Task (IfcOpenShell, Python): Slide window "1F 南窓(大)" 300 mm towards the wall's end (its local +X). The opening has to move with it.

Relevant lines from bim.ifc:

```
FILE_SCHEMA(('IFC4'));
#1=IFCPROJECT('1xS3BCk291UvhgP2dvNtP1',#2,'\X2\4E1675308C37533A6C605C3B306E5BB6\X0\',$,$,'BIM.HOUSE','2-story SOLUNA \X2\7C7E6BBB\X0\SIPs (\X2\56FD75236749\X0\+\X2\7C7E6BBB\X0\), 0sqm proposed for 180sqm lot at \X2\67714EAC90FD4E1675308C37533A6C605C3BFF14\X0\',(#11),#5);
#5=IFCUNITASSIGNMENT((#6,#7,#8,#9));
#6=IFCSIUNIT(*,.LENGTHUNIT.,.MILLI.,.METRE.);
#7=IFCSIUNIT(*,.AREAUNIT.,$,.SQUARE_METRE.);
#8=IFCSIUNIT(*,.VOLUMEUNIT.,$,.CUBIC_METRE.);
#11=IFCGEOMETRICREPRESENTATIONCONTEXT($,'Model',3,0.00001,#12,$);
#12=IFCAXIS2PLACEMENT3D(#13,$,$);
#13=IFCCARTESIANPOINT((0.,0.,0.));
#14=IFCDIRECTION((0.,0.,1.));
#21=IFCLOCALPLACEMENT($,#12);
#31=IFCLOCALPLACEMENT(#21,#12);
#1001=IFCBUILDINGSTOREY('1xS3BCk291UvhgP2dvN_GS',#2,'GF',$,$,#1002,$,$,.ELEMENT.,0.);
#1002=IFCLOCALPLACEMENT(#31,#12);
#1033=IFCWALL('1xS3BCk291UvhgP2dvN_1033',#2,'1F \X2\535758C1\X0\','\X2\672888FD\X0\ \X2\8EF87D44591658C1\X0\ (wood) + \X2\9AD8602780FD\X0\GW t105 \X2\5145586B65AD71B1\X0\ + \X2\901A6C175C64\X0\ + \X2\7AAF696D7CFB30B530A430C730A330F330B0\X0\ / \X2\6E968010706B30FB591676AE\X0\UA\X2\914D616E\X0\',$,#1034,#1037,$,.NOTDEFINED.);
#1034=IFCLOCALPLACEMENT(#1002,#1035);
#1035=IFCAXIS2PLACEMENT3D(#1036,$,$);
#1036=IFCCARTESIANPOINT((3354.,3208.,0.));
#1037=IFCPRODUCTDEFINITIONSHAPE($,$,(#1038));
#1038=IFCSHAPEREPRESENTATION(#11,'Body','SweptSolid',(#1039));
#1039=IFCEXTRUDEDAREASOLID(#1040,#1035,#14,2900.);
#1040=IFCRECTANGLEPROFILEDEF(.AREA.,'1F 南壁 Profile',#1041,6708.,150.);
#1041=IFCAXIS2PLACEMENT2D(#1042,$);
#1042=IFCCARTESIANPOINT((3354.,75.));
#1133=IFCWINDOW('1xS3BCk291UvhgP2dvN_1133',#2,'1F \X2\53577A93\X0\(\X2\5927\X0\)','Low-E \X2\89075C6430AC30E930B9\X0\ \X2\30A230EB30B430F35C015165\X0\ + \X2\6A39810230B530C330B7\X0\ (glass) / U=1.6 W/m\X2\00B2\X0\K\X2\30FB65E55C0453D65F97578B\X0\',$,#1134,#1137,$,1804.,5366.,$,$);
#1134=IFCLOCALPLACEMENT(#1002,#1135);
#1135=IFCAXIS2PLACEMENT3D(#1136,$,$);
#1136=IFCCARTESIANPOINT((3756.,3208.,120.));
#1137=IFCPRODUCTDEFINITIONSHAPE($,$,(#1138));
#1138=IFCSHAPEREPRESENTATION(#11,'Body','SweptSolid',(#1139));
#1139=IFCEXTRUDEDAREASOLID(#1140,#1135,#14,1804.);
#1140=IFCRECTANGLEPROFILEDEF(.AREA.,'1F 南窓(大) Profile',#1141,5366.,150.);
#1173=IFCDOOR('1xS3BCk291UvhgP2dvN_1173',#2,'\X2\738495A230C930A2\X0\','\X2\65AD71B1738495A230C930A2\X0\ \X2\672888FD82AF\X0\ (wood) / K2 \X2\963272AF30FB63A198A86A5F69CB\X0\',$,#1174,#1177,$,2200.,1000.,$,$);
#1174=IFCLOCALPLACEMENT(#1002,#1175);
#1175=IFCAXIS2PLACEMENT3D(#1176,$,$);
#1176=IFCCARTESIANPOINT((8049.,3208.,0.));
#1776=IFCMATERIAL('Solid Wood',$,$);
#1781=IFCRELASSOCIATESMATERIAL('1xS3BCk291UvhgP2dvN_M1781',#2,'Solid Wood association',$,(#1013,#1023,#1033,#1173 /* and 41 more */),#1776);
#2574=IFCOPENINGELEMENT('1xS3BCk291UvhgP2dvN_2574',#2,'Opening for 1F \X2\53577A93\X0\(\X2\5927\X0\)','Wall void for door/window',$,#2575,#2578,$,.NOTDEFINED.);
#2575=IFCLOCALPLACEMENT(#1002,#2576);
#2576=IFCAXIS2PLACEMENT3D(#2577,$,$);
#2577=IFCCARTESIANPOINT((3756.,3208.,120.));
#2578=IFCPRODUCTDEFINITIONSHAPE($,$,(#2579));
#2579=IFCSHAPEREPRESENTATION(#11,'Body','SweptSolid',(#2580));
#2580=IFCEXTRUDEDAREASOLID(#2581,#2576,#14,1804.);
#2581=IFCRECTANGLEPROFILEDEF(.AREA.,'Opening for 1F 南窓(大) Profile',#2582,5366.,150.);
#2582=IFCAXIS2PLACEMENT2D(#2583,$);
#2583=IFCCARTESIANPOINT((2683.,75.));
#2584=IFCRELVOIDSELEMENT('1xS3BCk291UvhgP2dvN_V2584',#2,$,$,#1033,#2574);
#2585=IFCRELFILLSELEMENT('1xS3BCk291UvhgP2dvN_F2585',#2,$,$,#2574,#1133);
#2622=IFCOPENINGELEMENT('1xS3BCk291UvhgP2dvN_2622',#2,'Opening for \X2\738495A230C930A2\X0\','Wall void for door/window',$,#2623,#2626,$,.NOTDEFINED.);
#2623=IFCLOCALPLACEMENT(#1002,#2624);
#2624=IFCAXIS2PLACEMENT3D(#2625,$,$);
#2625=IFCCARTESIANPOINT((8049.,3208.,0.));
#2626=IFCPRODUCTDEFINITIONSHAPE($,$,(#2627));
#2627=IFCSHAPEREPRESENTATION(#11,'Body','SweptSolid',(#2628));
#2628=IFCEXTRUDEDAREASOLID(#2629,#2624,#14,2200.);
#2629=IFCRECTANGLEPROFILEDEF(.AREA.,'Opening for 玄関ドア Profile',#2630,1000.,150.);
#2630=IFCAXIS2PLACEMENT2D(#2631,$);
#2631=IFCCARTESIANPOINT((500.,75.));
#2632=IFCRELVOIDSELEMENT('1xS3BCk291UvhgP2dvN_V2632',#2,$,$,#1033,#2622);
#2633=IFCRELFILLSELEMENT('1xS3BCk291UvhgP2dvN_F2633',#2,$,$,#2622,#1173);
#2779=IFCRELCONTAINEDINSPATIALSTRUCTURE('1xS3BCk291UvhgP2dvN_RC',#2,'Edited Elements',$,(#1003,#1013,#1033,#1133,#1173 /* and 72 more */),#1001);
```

```python
import ifcopenshell
import ifcopenshell.api.geometry
import ifcopenshell.util.placement
import ifcopenshell.util.unit

model = ifcopenshell.open("bim.ifc")
unit_scale = ifcopenshell.util.unit.calculate_unit_scale(model)

window = model.by_guid("1xS3BCk291UvhgP2dvN_1133")
opening = window.FillsVoids[0].RelatingOpeningElement
wall = opening.VoidsElements[0].RelatingBuildingElement

wall_matrix = ifcopenshell.util.placement.get_local_placement(wall.ObjectPlacement)
shift = wall_matrix[:3, 0] * 0.3 / unit_scale
before = ifcopenshell.util.placement.get_local_placement(window.ObjectPlacement)[:3, 3].copy()

# The window is not placed relative to its opening, so move both.
for product in (opening, window):
    matrix = ifcopenshell.util.placement.get_local_placement(product.ObjectPlacement)
    matrix[:3, 3] += shift
    ifcopenshell.api.geometry.edit_object_placement(model, product=product, matrix=matrix, is_si=False)

after = ifcopenshell.util.placement.get_local_placement(window.ObjectPlacement)[:3, 3]
print("window moved by", (after - before).round(3) + 0.0)

model.write("bim_updated.ifc")
```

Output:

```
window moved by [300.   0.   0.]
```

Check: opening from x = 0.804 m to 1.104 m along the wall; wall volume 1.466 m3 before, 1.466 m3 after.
